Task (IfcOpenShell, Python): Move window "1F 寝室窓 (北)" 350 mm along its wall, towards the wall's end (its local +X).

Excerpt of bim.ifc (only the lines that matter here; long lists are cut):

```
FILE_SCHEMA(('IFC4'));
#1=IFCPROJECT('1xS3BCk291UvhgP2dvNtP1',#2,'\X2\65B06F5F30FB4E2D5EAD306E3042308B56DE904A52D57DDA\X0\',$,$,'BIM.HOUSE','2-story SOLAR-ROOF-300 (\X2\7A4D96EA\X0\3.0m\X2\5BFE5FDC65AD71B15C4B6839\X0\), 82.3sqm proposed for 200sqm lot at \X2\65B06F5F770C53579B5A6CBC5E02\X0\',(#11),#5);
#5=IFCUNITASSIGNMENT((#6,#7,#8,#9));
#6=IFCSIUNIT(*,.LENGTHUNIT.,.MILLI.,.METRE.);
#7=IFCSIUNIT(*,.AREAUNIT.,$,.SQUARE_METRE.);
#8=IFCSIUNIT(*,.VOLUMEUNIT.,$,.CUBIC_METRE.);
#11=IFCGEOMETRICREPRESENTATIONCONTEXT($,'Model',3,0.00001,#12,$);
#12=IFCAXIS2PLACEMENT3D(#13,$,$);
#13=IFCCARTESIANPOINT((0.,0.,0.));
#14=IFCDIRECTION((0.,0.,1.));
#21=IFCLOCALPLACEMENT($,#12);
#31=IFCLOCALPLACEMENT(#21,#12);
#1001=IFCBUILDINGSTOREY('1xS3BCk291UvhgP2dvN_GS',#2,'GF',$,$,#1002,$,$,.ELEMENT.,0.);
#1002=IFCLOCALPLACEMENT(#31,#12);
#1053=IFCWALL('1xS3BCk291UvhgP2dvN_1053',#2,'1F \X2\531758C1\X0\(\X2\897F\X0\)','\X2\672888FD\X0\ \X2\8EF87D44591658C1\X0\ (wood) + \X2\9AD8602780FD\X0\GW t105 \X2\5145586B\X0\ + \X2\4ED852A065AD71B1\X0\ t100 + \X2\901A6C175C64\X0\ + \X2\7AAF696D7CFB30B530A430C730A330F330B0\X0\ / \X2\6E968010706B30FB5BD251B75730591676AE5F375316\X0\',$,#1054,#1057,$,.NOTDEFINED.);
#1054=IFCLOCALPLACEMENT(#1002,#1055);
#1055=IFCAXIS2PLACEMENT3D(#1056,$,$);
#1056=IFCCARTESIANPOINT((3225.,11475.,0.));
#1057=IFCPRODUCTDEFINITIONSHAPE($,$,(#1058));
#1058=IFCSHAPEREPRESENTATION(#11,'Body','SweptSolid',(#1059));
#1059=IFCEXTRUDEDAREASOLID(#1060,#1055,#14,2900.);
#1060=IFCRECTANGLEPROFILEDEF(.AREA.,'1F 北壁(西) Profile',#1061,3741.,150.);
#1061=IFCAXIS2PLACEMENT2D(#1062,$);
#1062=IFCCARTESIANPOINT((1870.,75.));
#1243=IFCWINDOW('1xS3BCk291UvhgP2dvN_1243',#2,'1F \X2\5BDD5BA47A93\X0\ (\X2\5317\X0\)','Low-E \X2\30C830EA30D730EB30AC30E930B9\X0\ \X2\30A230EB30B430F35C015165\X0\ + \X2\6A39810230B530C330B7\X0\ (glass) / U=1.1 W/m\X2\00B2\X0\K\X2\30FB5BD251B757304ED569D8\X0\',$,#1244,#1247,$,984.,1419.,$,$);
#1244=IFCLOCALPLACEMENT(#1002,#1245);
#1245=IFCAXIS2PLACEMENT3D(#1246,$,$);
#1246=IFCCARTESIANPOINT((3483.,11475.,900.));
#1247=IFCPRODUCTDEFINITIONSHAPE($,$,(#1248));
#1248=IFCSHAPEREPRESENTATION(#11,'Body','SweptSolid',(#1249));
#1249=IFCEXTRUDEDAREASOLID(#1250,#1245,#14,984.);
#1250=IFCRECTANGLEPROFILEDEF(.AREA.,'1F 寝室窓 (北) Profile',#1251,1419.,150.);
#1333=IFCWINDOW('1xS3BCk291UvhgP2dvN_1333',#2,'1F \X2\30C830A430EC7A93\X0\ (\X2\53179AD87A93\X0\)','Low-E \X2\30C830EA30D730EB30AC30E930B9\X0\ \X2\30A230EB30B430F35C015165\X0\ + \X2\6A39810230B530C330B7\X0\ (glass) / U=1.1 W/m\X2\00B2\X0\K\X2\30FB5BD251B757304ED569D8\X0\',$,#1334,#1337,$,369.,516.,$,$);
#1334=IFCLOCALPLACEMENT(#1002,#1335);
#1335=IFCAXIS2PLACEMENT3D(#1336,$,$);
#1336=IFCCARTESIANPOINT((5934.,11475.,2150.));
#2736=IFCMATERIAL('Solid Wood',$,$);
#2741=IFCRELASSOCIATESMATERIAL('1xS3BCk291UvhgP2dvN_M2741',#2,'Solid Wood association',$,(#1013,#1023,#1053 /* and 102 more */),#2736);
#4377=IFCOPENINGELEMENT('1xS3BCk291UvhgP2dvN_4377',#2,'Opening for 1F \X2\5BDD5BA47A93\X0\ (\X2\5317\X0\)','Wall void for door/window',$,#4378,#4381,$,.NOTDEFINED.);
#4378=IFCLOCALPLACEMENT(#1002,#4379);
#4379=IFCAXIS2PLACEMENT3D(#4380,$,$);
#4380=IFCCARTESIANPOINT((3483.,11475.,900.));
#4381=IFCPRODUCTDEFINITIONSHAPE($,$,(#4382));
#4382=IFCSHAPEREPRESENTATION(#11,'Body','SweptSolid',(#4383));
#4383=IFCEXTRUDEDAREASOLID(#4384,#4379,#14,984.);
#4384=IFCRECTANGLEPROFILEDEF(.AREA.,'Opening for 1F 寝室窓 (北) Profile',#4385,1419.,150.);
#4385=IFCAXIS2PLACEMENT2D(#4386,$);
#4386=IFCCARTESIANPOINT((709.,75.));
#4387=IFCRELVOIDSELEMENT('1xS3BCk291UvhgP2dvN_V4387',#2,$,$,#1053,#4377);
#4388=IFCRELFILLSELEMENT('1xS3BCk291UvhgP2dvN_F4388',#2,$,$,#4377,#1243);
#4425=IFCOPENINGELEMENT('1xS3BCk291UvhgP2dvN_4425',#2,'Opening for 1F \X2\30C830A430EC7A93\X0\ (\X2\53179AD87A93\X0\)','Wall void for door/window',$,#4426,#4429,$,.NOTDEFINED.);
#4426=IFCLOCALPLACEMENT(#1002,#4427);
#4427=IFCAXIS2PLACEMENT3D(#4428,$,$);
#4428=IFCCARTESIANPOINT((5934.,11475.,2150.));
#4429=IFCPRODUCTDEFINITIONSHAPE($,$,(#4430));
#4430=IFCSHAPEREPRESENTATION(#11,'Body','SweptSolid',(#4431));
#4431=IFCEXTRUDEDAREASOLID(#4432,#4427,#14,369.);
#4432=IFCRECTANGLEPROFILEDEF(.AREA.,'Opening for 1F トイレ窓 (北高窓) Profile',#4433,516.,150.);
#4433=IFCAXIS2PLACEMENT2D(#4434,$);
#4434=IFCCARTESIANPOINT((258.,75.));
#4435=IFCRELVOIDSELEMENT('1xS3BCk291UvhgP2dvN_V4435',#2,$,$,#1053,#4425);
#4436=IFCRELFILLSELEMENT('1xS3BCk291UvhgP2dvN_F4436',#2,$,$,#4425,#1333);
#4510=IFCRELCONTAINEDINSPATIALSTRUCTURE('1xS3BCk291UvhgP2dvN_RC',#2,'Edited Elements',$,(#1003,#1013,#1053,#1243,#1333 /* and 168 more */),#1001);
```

```python
import ifcopenshell
import ifcopenshell.api.geometry
import ifcopenshell.util.placement
import ifcopenshell.util.unit

model = ifcopenshell.open("bim.ifc")
unit_scale = ifcopenshell.util.unit.calculate_unit_scale(model)

window = model.by_guid("1xS3BCk291UvhgP2dvN_1243")
opening = window.FillsVoids[0].RelatingOpeningElement
wall = opening.VoidsElements[0].RelatingBuildingElement

wall_matrix = ifcopenshell.util.placement.get_local_placement(wall.ObjectPlacement)
shift = wall_matrix[:3, 0] * 0.35 / unit_scale
before = ifcopenshell.util.placement.get_local_placement(window.ObjectPlacement)[:3, 3].copy()

# The window is not placed relative to its opening, so move both.
for product in (opening, window):
    matrix = ifcopenshell.util.placement.get_local_placement(product.ObjectPlacement)
    matrix[:3, 3] += shift
    ifcopenshell.api.geometry.edit_object_placement(model, product=product, matrix=matrix, is_si=False)

after = ifcopenshell.util.placement.get_local_placement(window.ObjectPlacement)[:3, 3]
print("window moved by", (after - before).round(3) + 0.0)

model.write("bim_v2.ifc")
```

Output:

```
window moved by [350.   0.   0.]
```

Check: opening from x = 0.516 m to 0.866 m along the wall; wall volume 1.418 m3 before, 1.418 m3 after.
